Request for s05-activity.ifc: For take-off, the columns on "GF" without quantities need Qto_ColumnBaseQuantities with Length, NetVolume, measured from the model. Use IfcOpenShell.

First a look at what the model holds.

```python
import ifcopenshell
import ifcopenshell.util.element
import ifcopenshell.util.unit

model = ifcopenshell.open("s05-activity.ifc")
print(model.schema)
for unit_type in ("LENGTHUNIT", "AREAUNIT", "VOLUMEUNIT"):
    print(unit_type, ifcopenshell.util.unit.calculate_unit_scale(model, unit_type))
storey = next(s for s in model.by_type("IfcBuildingStorey") if s.Name == "GF")
columns = [e for e in ifcopenshell.util.element.get_decomposition(storey) if e.is_a("IfcColumn")]
for e in sorted(columns, key=lambda e: e.id()):
    print(e.id(), e.is_a(), e.Name, list(ifcopenshell.util.element.get_psets(e, qtos_only=True)), sep=" | ")
```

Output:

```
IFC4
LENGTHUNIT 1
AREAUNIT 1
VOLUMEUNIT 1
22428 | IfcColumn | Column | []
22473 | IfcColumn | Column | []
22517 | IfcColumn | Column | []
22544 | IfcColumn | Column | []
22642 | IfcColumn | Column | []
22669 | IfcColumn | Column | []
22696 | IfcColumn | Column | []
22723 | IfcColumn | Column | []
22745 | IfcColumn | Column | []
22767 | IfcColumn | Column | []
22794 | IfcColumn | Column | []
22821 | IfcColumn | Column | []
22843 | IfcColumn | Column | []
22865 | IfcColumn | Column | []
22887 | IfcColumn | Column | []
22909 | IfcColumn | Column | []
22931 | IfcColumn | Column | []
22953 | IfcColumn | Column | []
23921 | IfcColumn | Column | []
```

```python
import ifcopenshell
import ifcopenshell.api.pset
import ifcopenshell.geom
import ifcopenshell.util.element
import ifcopenshell.util.shape
import ifcopenshell.util.unit

model = ifcopenshell.open("s05-activity.ifc")
unit_scale = ifcopenshell.util.unit.calculate_unit_scale(model)
volume_scale = ifcopenshell.util.unit.calculate_unit_scale(model, "VOLUMEUNIT")
settings = ifcopenshell.geom.settings()

storey = next(s for s in model.by_type("IfcBuildingStorey") if s.Name == "GF")
columns = [e for e in ifcopenshell.util.element.get_decomposition(storey) if e.is_a("IfcColumn")]

for e in sorted(columns, key=lambda e: e.id()):
    if ifcopenshell.util.element.get_psets(e, qtos_only=True, should_inherit=False):
        continue
    # Geometry comes back in metres, in the element's own axes.
    shape = ifcopenshell.geom.create_shape(settings, e)
    values = {
        "Length": ifcopenshell.util.shape.get_z(shape.geometry) / unit_scale,
        "NetVolume": ifcopenshell.util.shape.get_volume(shape.geometry) / volume_scale,
    }
    qto = ifcopenshell.api.pset.add_qto(model, product=e, name="Qto_ColumnBaseQuantities")
    ifcopenshell.api.pset.edit_qto(model, qto=qto, properties=values)
    print(e.id(), {k: round(v, 3) for k, v in values.items()})

model.write("s05-activity_rev.ifc")
```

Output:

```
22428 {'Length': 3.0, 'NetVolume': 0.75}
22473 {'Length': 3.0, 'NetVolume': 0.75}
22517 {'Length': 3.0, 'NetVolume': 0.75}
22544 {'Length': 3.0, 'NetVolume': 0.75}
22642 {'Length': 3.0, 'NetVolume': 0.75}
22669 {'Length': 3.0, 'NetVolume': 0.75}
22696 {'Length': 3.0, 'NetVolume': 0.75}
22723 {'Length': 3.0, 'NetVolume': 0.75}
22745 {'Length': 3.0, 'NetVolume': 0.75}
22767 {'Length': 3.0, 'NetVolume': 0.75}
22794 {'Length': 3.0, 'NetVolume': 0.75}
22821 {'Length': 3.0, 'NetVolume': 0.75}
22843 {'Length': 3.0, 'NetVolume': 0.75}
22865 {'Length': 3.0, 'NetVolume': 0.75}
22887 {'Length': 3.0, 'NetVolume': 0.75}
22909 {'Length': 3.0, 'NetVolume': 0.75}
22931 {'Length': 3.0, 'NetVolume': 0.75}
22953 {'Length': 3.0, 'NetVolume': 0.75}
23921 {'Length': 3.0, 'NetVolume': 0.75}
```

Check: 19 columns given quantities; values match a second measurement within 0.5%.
